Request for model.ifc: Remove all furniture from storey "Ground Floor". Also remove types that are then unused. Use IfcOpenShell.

First a look at what the model holds.

```python
import ifcopenshell
import ifcopenshell.util.element

model = ifcopenshell.open("model.ifc")
print(model.schema)
storey = next(s for s in model.by_type("IfcBuildingStorey") if s.Name == "Ground Floor")
furniture = [e for e in ifcopenshell.util.element.get_decomposition(storey) if e.is_a("IfcFurnishingElement")]
seen = {}
for e in furniture:
    element_type = ifcopenshell.util.element.get_type(e)
    name = element_type.Name if element_type not in (None, e) else None
    seen[name] = seen.get(name, 0) + 1
for name, count in sorted(seen.items(), key=str):
    print(count, "x", name)
```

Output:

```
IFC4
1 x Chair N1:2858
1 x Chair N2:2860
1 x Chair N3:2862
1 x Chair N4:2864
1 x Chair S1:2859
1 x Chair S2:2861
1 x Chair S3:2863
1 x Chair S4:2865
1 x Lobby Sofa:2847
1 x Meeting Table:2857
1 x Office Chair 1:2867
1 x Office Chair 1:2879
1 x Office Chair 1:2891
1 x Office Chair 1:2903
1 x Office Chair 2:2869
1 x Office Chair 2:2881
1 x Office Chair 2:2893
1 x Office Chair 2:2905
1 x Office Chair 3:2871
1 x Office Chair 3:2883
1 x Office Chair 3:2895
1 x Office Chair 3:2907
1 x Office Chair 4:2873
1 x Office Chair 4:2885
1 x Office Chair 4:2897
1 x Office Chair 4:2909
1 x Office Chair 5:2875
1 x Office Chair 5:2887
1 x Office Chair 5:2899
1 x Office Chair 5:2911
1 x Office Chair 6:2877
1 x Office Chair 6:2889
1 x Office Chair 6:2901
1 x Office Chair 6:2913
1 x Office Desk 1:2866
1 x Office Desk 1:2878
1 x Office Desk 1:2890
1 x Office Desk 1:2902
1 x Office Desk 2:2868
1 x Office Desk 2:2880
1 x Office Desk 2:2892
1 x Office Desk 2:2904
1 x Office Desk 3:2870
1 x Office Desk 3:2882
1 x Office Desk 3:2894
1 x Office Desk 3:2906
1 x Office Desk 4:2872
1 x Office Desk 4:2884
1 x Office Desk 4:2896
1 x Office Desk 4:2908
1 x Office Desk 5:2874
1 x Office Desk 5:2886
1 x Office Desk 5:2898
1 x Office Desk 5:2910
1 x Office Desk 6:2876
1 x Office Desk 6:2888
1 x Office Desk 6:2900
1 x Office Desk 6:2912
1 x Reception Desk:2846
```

```python
import ifcopenshell
import ifcopenshell.api.root
import ifcopenshell.util.element

model = ifcopenshell.open("model.ifc")

storey = next(s for s in model.by_type("IfcBuildingStorey") if s.Name == "Ground Floor")
furniture = [e for e in ifcopenshell.util.element.get_decomposition(storey) if e.is_a("IfcFurnishingElement")]
types = {ifcopenshell.util.element.get_type(e) for e in furniture} - {None, *furniture}

for e in furniture:
    ifcopenshell.api.root.remove_product(model, product=e)
print(len(furniture), "removed")

unused = [t for t in types if not ifcopenshell.util.element.get_types(t)]
for t in unused:
    ifcopenshell.api.root.remove_product(model, product=t)
print(len(unused), "unused types removed")

model.write("model-out.ifc")
```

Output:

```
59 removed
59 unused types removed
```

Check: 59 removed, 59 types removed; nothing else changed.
